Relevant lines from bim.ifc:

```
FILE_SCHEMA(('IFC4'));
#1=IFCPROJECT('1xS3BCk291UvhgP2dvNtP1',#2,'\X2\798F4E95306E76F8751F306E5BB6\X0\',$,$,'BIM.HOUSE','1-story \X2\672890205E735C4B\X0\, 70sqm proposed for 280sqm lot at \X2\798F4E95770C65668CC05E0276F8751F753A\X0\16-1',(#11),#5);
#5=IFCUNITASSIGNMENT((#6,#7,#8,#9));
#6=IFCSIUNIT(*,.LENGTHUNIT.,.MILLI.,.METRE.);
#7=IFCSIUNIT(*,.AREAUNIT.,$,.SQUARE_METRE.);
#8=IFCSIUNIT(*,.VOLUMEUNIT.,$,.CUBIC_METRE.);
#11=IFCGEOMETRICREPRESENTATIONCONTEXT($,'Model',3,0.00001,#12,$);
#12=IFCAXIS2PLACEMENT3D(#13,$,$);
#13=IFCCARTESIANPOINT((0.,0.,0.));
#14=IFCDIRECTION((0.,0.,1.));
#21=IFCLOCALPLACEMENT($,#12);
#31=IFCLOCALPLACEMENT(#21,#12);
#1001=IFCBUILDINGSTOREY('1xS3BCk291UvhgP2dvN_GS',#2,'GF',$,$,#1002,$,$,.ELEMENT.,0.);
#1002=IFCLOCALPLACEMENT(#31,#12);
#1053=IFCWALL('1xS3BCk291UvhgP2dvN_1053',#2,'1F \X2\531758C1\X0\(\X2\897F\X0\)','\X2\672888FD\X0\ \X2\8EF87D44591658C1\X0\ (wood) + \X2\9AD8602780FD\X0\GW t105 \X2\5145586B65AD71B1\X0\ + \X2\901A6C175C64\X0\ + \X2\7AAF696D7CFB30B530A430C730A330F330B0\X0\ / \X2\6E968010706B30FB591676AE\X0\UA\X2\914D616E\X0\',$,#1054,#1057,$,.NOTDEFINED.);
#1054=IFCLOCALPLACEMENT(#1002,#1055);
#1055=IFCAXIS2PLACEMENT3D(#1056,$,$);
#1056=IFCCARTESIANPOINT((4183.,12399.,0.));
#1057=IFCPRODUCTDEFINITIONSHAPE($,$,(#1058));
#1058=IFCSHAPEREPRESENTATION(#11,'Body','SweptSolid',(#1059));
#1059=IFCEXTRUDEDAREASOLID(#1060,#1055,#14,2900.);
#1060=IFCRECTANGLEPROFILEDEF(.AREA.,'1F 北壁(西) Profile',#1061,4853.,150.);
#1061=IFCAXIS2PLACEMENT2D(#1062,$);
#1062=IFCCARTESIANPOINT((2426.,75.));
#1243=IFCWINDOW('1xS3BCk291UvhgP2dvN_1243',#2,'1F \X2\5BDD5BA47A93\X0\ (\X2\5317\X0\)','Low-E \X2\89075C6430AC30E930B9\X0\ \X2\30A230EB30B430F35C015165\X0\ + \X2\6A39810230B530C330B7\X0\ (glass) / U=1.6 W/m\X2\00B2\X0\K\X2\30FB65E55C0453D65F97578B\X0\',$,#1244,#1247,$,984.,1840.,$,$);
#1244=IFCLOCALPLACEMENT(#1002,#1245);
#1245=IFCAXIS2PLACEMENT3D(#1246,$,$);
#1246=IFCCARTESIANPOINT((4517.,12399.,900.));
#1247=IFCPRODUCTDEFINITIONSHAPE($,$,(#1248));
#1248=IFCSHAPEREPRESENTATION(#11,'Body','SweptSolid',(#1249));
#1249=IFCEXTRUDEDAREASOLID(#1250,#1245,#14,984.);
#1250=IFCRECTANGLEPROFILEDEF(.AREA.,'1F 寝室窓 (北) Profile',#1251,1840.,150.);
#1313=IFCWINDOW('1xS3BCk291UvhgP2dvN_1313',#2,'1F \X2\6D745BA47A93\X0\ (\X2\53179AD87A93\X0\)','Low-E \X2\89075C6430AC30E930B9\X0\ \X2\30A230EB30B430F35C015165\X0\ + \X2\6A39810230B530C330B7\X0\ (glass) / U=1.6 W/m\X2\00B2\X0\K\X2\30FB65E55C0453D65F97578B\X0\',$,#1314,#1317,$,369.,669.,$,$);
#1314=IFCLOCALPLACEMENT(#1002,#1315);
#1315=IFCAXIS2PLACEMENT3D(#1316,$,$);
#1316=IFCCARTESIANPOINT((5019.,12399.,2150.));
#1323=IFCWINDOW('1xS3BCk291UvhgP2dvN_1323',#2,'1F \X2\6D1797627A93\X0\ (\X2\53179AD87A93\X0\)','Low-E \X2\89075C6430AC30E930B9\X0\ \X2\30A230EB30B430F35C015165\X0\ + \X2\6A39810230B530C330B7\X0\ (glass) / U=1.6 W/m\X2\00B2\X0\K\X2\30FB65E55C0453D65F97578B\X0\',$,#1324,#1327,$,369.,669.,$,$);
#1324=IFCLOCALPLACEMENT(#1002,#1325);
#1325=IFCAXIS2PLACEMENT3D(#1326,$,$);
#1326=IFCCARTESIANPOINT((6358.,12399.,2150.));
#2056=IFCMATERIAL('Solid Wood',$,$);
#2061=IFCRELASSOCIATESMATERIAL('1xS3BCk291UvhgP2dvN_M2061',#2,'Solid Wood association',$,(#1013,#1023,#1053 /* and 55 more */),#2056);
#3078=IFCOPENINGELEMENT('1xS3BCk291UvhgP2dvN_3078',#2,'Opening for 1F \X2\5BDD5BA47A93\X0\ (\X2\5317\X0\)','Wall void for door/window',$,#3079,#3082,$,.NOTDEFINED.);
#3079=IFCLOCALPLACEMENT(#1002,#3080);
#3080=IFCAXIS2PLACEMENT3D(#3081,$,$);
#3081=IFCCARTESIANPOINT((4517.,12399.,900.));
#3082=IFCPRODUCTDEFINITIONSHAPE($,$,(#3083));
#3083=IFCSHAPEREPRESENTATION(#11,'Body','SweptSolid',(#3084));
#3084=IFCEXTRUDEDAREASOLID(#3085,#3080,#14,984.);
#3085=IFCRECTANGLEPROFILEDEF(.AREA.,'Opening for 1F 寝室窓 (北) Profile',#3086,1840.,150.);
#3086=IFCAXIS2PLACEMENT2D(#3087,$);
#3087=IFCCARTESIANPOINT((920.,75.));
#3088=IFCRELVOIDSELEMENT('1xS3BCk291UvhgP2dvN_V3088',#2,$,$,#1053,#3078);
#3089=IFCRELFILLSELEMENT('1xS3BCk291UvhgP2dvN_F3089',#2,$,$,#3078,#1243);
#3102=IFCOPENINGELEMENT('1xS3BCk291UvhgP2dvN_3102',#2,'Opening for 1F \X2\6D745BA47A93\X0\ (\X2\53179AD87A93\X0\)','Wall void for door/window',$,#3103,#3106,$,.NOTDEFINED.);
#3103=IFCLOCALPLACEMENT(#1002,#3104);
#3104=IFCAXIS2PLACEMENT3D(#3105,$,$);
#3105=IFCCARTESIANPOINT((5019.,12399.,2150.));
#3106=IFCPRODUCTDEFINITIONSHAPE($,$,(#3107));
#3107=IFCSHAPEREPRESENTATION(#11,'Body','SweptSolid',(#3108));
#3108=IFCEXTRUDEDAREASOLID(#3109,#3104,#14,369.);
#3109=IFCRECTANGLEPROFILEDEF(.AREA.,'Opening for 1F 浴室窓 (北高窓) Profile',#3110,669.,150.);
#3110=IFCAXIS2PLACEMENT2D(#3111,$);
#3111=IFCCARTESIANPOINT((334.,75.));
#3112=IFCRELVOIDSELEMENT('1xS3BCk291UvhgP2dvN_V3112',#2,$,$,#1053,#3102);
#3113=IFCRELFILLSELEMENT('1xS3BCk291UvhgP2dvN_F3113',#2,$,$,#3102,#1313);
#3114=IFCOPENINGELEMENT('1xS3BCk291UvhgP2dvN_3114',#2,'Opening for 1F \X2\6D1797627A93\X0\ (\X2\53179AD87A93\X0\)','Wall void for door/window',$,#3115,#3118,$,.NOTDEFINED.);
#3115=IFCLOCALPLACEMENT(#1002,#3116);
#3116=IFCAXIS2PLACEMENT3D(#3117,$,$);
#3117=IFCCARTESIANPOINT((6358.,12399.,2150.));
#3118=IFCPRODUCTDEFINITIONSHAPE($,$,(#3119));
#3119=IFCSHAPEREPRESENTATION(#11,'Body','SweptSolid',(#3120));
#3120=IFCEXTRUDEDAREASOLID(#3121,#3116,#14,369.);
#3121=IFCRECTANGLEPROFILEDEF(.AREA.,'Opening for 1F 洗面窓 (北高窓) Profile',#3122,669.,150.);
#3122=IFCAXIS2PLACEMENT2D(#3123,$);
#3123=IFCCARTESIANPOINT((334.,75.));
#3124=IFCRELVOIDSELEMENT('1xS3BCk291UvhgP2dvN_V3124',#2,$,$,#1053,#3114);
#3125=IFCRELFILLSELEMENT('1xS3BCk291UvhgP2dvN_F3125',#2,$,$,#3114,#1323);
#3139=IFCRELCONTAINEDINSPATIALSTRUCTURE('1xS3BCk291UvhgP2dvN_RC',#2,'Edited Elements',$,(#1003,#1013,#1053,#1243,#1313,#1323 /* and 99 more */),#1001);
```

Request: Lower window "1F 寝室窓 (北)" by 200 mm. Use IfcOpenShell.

```python
import numpy as np
import ifcopenshell
import ifcopenshell.api.geometry
import ifcopenshell.util.placement
import ifcopenshell.util.unit

model = ifcopenshell.open("bim.ifc")
unit_scale = ifcopenshell.util.unit.calculate_unit_scale(model)

window = model.by_guid("1xS3BCk291UvhgP2dvN_1243")
opening = window.FillsVoids[0].RelatingOpeningElement
dz = -200.0

shift = np.array([0.0, 0.0, dz])
# The window is not placed relative to its opening, so move both.
for product in (opening, window):
    matrix = ifcopenshell.util.placement.get_local_placement(product.ObjectPlacement)
    matrix[:3, 3] += shift
    ifcopenshell.api.geometry.edit_object_placement(model, product=product, matrix=matrix, is_si=False)

print(f"moved by {dz * unit_scale:+.3f} m")

model.write("bim-out.ifc")
```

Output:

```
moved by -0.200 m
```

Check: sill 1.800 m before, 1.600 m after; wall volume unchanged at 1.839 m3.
